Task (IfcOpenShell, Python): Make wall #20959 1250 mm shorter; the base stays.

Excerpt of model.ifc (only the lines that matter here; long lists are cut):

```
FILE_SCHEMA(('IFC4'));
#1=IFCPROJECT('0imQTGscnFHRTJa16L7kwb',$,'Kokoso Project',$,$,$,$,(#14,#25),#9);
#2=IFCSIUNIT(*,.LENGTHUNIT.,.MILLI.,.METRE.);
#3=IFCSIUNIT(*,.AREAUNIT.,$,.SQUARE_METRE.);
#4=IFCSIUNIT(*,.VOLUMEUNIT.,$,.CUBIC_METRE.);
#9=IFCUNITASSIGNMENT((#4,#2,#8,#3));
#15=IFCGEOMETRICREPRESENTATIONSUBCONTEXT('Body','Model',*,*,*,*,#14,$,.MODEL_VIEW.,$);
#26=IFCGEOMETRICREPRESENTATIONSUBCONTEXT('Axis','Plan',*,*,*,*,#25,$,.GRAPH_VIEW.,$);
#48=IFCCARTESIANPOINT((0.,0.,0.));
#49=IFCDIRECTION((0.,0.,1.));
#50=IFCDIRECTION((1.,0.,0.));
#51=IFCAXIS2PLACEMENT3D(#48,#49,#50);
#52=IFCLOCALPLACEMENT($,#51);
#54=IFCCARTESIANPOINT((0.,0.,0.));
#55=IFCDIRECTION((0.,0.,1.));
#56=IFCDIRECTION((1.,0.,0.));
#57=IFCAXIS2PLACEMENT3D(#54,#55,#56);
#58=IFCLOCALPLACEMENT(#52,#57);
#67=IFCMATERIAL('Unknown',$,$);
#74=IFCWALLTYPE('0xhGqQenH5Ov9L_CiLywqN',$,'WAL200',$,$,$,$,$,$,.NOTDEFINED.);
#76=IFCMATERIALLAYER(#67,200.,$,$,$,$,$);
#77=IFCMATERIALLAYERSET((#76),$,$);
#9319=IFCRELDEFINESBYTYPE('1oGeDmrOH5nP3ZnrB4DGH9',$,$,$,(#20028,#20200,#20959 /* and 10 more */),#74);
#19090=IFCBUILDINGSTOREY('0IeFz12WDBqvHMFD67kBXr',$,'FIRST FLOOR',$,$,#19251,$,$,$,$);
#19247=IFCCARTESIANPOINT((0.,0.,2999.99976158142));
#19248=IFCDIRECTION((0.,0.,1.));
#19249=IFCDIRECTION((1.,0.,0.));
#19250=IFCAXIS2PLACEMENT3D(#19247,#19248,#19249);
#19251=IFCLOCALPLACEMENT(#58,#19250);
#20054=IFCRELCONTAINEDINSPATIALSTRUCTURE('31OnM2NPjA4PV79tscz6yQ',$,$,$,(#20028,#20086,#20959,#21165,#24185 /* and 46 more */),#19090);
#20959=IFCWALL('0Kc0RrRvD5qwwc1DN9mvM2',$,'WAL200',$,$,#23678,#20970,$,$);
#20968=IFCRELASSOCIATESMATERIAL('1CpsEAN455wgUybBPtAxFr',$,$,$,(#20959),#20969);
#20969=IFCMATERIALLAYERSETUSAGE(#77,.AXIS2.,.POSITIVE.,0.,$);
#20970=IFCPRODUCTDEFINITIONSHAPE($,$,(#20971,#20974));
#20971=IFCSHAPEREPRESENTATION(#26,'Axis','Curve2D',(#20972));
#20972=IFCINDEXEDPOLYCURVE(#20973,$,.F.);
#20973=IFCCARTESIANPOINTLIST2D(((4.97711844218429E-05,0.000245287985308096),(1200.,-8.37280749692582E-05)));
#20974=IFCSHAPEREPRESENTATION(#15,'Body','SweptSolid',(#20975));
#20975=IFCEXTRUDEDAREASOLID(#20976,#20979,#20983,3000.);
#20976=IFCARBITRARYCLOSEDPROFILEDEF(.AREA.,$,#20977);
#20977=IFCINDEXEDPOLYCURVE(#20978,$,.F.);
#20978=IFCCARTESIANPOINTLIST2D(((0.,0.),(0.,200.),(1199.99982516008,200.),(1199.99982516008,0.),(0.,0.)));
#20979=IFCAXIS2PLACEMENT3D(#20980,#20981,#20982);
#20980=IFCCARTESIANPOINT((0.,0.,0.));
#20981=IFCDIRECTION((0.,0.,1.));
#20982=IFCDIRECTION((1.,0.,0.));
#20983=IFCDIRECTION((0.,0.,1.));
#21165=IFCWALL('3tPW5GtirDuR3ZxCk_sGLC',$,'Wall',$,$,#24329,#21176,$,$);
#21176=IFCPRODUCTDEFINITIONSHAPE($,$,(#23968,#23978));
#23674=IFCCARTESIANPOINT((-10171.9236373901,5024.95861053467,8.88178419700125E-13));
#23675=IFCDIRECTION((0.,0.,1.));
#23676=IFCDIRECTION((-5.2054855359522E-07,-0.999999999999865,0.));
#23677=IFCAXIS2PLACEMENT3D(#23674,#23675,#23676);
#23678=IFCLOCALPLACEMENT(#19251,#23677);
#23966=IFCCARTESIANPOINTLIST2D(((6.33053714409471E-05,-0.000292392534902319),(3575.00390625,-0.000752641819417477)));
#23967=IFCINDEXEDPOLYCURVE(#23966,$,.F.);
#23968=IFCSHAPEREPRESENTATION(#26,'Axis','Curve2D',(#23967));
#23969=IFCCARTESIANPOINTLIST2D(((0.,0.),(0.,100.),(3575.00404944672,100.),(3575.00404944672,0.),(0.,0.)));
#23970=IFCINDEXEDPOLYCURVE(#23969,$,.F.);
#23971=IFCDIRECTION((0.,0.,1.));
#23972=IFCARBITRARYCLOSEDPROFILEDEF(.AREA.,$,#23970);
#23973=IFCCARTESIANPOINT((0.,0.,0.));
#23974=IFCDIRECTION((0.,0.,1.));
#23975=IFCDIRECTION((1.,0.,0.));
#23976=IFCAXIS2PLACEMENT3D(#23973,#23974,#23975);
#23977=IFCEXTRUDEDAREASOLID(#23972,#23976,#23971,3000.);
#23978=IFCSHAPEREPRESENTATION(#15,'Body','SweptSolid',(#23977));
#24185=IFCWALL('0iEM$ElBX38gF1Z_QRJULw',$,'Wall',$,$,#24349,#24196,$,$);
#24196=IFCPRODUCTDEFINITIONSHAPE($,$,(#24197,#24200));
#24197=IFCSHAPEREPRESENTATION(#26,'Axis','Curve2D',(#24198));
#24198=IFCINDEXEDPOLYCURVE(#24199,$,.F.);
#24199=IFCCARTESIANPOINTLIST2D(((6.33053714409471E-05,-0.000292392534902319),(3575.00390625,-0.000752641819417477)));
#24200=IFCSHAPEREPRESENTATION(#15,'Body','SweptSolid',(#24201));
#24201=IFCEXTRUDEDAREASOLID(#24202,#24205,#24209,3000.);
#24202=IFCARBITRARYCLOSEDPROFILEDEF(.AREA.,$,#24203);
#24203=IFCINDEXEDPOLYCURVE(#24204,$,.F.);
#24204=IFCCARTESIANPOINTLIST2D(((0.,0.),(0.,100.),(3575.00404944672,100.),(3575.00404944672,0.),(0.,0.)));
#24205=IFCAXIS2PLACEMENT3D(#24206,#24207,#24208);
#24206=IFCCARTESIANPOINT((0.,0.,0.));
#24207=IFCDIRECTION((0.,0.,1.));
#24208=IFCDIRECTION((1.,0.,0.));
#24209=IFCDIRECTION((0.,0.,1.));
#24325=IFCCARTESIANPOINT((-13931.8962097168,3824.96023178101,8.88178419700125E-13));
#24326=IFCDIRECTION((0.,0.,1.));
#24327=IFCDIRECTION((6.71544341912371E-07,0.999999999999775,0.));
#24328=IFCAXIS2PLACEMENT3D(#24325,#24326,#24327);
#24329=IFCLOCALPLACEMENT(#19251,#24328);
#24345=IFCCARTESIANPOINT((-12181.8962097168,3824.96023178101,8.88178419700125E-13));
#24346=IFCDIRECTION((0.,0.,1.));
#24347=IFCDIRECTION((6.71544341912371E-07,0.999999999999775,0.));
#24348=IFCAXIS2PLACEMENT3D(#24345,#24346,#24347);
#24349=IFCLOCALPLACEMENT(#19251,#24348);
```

```python
import ifcopenshell
import ifcopenshell.geom
import ifcopenshell.util.representation
import ifcopenshell.util.shape

model = ifcopenshell.open("model.ifc")
settings = ifcopenshell.geom.settings()


def volume(element):
    """Net volume in cubic metres, openings subtracted."""
    shape = ifcopenshell.geom.create_shape(settings, element)
    return ifcopenshell.util.shape.get_volume(shape.geometry)


wall = model.by_guid("0Kc0RrRvD5qwwc1DN9mvM2")
before = volume(wall)

body = ifcopenshell.util.representation.get_representation(wall, "Model", "Body")
solid = body.Items[0]
old_height = solid.Depth
solid.Depth -= 1250.0
after = volume(wall)

print(f"height {old_height:g} -> {solid.Depth:g}, volume {before:.3f} -> {after:.3f} m3")

model.write("model_v2.ifc")
```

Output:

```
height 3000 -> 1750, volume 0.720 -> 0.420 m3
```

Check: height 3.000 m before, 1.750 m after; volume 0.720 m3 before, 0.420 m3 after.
